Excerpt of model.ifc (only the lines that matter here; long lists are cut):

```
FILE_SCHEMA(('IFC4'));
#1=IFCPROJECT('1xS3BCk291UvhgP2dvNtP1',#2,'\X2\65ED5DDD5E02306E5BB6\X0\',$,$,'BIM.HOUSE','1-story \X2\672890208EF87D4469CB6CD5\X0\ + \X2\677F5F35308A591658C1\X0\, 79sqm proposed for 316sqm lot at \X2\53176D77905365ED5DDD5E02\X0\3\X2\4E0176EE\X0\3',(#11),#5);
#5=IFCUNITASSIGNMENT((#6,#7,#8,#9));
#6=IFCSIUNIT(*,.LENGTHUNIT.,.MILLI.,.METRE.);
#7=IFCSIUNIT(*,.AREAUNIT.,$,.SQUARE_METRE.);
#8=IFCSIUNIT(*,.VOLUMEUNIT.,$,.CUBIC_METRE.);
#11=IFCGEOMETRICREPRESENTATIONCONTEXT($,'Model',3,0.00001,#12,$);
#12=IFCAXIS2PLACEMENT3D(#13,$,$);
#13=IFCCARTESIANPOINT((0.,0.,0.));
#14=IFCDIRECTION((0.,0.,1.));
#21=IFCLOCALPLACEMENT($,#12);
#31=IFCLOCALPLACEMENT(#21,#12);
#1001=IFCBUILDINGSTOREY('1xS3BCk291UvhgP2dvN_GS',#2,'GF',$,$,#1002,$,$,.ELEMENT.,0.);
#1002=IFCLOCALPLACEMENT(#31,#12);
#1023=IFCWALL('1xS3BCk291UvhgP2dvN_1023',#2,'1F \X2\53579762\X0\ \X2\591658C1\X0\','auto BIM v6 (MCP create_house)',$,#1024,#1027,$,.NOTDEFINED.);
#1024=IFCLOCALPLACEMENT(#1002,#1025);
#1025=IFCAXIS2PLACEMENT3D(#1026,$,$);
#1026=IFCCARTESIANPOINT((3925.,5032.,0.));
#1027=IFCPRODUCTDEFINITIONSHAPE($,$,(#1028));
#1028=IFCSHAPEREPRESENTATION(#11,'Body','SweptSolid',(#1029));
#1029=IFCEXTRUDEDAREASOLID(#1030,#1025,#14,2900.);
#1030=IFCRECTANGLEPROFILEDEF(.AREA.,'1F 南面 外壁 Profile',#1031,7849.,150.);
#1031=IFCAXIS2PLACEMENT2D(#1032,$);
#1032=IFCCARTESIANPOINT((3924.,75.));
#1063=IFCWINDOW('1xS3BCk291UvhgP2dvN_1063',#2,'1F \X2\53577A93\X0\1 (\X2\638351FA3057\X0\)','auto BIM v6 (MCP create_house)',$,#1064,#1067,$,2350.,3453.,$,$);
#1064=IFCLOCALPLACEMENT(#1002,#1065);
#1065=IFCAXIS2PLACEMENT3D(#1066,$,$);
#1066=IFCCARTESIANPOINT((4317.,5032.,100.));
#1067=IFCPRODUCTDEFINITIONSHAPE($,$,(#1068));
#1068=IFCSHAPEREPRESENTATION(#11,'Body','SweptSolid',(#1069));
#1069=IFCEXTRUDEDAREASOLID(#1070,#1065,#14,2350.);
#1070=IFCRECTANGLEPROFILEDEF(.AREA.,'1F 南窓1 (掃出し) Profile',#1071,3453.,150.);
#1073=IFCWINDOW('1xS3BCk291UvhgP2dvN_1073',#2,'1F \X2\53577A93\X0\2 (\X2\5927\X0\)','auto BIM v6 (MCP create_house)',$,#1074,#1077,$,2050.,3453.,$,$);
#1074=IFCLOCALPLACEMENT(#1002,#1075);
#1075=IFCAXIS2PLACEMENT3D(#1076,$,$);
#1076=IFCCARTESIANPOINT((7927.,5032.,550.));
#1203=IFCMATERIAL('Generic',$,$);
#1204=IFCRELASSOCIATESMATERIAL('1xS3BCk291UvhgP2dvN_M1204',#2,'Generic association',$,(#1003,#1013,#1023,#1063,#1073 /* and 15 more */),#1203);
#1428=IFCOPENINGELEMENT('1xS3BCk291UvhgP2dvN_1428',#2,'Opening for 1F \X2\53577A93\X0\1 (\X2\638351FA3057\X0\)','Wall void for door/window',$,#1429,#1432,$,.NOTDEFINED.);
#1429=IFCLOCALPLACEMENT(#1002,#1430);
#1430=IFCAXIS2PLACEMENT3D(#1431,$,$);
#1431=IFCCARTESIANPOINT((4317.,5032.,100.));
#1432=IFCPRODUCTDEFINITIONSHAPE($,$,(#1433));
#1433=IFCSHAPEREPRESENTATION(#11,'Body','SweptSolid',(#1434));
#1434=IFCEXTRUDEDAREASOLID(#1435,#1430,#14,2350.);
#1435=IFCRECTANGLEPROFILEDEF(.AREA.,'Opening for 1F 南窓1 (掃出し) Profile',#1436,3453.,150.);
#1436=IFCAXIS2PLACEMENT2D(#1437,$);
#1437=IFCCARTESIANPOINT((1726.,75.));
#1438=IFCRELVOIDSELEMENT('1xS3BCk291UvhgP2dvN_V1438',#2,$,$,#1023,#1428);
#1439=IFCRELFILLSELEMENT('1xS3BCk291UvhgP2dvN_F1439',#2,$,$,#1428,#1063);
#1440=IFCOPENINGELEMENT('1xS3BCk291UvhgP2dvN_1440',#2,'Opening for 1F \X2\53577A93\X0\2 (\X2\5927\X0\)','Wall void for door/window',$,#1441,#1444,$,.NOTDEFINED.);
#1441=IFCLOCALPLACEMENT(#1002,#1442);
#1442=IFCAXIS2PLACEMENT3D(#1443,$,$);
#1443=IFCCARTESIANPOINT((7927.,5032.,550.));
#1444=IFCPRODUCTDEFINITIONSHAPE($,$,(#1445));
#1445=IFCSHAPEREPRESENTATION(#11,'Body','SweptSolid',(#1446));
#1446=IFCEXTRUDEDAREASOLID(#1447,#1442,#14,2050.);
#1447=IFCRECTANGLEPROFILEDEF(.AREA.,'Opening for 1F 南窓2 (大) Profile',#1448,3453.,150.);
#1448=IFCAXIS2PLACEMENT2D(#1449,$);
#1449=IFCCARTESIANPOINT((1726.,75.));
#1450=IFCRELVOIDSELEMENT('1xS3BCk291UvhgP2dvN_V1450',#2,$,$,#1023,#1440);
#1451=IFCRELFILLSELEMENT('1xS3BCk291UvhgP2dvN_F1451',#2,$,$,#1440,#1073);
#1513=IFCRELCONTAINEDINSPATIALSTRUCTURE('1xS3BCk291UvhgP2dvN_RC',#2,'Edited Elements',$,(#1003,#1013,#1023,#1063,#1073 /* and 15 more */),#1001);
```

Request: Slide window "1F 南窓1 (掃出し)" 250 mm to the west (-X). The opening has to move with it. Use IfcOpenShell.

```python
import ifcopenshell
import ifcopenshell.api.geometry
import ifcopenshell.util.placement
import ifcopenshell.util.unit

model = ifcopenshell.open("model.ifc")
unit_scale = ifcopenshell.util.unit.calculate_unit_scale(model)

window = model.by_guid("1xS3BCk291UvhgP2dvN_1063")
opening = window.FillsVoids[0].RelatingOpeningElement
wall = opening.VoidsElements[0].RelatingBuildingElement

wall_matrix = ifcopenshell.util.placement.get_local_placement(wall.ObjectPlacement)
shift = wall_matrix[:3, 0] * -0.25 / unit_scale
before = ifcopenshell.util.placement.get_local_placement(window.ObjectPlacement)[:3, 3].copy()

# The window is not placed relative to its opening, so move both.
for product in (opening, window):
    matrix = ifcopenshell.util.placement.get_local_placement(product.ObjectPlacement)
    matrix[:3, 3] += shift
    ifcopenshell.api.geometry.edit_object_placement(model, product=product, matrix=matrix, is_si=False)

after = ifcopenshell.util.placement.get_local_placement(window.ObjectPlacement)[:3, 3]
print("window moved by", (after - before).round(3) + 0.0)

model.write("model_v2.ifc")
```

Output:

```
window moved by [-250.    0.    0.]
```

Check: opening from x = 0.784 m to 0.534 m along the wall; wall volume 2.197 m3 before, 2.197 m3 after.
